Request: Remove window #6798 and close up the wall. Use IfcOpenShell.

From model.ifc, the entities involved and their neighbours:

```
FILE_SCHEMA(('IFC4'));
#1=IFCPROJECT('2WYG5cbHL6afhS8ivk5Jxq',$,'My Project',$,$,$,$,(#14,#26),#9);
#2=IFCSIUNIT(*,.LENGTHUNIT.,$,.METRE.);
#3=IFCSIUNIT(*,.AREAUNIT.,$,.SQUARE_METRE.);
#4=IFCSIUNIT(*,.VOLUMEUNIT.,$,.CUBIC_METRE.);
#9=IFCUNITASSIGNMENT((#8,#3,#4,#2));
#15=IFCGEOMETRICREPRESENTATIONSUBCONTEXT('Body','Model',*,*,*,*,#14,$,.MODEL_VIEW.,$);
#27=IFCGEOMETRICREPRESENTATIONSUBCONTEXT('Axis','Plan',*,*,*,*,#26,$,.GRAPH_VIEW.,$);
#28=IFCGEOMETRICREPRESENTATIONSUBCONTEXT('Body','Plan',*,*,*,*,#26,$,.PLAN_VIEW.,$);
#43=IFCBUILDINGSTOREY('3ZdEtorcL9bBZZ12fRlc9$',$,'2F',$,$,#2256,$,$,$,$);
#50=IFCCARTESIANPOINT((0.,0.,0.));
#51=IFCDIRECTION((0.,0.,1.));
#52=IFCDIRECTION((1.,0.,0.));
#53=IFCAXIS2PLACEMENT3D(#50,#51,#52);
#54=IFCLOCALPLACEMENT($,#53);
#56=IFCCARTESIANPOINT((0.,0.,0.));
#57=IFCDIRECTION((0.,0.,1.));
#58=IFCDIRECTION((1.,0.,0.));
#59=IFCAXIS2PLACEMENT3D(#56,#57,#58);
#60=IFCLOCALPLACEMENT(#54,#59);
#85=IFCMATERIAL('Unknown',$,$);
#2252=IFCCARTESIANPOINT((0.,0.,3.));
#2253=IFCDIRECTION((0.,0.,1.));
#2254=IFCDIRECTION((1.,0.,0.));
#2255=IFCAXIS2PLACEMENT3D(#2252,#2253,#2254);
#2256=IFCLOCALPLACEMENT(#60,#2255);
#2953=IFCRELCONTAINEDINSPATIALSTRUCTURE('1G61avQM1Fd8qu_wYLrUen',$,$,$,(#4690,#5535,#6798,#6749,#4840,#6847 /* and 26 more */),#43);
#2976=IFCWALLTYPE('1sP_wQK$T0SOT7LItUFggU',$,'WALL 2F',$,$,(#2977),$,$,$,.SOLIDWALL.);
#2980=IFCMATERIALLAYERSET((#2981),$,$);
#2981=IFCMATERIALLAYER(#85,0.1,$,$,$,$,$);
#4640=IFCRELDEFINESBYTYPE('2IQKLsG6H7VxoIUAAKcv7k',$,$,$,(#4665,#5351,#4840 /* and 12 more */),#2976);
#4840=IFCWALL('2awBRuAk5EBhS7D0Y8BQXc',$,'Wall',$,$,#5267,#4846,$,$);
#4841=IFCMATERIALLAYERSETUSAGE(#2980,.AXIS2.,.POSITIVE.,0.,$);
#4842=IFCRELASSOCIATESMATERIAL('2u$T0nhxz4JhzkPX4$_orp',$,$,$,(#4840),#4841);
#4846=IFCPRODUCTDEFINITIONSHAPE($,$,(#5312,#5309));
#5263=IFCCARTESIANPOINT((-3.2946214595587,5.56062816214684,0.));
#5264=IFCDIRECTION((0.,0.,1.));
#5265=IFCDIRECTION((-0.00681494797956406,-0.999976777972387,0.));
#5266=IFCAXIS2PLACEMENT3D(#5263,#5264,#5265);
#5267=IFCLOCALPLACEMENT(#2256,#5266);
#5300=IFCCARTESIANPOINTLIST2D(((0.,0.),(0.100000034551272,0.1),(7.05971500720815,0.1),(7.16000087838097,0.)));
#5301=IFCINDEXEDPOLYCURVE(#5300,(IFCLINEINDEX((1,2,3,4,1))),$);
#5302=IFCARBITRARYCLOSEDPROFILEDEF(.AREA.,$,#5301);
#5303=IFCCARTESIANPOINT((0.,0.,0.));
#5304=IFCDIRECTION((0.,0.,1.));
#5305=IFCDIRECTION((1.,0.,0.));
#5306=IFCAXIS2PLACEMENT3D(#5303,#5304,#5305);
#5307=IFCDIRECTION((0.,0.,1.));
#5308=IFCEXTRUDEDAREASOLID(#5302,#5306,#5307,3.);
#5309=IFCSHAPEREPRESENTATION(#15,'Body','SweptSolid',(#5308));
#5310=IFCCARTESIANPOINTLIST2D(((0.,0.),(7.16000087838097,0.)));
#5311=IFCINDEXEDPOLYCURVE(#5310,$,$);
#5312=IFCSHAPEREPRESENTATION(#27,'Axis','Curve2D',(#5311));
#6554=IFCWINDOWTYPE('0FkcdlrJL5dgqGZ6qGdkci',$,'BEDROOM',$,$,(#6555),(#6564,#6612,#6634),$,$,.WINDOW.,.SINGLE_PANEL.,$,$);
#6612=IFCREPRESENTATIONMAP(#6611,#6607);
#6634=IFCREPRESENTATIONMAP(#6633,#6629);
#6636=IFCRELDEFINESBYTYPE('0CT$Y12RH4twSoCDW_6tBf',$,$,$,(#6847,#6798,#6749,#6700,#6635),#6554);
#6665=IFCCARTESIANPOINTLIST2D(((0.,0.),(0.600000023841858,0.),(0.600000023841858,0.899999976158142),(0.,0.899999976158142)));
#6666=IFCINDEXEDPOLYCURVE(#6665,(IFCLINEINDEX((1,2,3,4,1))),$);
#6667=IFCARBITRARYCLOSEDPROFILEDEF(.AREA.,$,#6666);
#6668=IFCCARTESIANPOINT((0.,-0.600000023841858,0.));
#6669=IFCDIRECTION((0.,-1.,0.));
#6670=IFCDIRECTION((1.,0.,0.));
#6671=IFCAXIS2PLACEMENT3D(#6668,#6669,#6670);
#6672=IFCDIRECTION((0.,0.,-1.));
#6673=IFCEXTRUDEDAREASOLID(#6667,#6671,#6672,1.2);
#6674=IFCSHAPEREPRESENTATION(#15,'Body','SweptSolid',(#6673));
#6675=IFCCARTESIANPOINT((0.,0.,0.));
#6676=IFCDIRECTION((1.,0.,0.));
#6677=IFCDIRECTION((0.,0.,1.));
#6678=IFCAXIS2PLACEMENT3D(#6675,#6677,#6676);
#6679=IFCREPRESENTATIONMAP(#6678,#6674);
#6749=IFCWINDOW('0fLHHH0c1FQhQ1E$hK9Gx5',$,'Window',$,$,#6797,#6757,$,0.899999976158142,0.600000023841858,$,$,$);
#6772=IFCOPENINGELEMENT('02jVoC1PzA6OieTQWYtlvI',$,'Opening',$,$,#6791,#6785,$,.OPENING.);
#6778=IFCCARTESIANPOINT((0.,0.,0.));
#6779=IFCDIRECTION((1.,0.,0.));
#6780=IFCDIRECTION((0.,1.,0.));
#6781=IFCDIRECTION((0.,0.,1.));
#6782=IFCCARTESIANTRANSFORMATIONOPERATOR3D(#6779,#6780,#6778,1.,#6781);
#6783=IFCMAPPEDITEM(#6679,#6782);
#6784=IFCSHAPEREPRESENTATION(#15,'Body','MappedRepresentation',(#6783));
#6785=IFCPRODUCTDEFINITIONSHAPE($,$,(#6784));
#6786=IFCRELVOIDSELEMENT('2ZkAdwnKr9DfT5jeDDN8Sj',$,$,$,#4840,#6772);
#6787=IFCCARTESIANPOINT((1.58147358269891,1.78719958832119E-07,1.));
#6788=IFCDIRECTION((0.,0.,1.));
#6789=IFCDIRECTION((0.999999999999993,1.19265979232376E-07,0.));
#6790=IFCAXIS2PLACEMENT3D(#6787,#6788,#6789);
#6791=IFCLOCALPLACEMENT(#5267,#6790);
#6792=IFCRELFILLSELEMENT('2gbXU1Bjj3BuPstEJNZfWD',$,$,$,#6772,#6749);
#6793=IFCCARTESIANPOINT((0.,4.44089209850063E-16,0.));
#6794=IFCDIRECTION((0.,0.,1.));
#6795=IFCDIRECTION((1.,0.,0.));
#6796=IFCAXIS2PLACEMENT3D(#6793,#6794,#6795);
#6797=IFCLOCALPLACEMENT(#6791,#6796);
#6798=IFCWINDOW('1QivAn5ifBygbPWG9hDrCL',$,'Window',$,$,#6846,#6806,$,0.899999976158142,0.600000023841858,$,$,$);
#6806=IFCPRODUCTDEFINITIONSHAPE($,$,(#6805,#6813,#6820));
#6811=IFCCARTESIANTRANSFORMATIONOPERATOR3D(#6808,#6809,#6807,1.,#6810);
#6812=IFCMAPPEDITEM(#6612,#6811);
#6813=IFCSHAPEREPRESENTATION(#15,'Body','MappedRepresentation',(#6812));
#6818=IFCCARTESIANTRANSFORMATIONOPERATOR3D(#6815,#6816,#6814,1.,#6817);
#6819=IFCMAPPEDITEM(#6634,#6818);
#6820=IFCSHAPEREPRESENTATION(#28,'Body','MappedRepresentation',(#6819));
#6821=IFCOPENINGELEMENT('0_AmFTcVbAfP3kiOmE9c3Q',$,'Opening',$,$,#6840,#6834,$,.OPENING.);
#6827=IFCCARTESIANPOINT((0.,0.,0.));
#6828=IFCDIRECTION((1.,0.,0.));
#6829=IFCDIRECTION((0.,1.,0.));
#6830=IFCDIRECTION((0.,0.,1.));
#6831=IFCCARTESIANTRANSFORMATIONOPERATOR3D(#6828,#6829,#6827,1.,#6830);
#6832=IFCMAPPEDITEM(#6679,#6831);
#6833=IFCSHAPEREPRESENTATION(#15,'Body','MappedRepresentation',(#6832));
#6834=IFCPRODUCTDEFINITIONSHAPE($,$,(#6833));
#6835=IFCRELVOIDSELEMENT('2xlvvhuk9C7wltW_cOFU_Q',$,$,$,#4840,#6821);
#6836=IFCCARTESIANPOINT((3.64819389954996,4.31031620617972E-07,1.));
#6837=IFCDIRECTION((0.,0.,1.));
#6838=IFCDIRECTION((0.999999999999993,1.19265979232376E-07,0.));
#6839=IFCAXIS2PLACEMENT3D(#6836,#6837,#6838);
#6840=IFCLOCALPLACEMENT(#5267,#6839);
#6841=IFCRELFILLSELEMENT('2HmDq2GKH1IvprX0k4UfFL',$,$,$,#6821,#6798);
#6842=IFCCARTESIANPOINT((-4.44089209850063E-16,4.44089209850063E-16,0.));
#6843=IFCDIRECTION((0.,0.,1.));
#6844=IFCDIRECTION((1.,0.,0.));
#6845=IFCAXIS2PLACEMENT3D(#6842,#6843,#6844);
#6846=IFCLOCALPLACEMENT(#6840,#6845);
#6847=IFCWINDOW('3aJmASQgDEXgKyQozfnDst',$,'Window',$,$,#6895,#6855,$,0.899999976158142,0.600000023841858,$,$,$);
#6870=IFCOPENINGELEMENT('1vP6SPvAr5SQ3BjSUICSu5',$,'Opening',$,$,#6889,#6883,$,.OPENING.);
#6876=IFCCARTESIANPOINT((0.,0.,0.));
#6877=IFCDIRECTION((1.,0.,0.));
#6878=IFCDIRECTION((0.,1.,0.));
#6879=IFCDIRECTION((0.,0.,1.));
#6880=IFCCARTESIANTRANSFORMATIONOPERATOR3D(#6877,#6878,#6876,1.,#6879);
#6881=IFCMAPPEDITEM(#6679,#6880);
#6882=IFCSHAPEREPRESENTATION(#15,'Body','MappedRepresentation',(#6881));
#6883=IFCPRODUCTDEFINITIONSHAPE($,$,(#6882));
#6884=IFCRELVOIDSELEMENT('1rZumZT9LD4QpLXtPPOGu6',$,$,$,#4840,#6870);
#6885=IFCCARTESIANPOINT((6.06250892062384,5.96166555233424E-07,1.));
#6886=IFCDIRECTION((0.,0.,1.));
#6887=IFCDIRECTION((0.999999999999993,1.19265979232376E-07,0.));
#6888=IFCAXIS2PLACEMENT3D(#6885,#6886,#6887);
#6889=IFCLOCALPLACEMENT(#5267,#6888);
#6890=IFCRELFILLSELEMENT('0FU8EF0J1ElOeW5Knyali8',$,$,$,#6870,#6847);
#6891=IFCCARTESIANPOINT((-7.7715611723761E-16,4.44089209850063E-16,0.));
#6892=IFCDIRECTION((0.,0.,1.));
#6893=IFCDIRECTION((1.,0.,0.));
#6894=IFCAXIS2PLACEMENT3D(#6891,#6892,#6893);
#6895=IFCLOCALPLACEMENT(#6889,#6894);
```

```python
import ifcopenshell
import ifcopenshell.api.feature
import ifcopenshell.api.root
import ifcopenshell.geom
import ifcopenshell.util.shape

model = ifcopenshell.open("model.ifc")
settings = ifcopenshell.geom.settings()


def volume(element):
    """Net volume in cubic metres, openings subtracted."""
    shape = ifcopenshell.geom.create_shape(settings, element)
    return ifcopenshell.util.shape.get_volume(shape.geometry)


window = model.by_guid("1QivAn5ifBygbPWG9hDrCL")
opening = window.FillsVoids[0].RelatingOpeningElement
wall = opening.VoidsElements[0].RelatingBuildingElement
before = volume(wall)

ifcopenshell.api.root.remove_product(model, product=window)
ifcopenshell.api.feature.remove_feature(model, feature=opening)

after = volume(wall)

print(f"wall volume {before:.3f} -> {after:.3f} m3")

model.write("model-out.ifc")
```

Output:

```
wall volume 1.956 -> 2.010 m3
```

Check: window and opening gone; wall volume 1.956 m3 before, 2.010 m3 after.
